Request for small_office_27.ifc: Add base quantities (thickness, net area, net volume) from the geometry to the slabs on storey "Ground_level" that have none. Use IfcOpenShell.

First a look at what the model holds.

```python
import ifcopenshell
import ifcopenshell.util.element
import ifcopenshell.util.unit

model = ifcopenshell.open("small_office_27.ifc")
print(model.schema)
for unit_type in ("LENGTHUNIT", "AREAUNIT", "VOLUMEUNIT"):
    print(unit_type, ifcopenshell.util.unit.calculate_unit_scale(model, unit_type))
storey = next(s for s in model.by_type("IfcBuildingStorey") if s.Name == "Ground_level")
slabs = [e for e in ifcopenshell.util.element.get_decomposition(storey) if e.is_a("IfcSlab")]
for e in sorted(slabs, key=lambda e: e.id()):
    print(e.id(), e.is_a(), e.Name, list(ifcopenshell.util.element.get_psets(e, qtos_only=True)), sep=" | ")
```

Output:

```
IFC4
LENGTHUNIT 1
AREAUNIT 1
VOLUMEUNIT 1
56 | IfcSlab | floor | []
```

```python
import ifcopenshell
import ifcopenshell.api.pset
import ifcopenshell.geom
import ifcopenshell.util.element
import ifcopenshell.util.shape
import ifcopenshell.util.unit

model = ifcopenshell.open("small_office_27.ifc")
unit_scale = ifcopenshell.util.unit.calculate_unit_scale(model)
area_scale = ifcopenshell.util.unit.calculate_unit_scale(model, "AREAUNIT")
volume_scale = ifcopenshell.util.unit.calculate_unit_scale(model, "VOLUMEUNIT")
settings = ifcopenshell.geom.settings()

storey = next(s for s in model.by_type("IfcBuildingStorey") if s.Name == "Ground_level")
slabs = [e for e in ifcopenshell.util.element.get_decomposition(storey) if e.is_a("IfcSlab")]

for e in sorted(slabs, key=lambda e: e.id()):
    if ifcopenshell.util.element.get_psets(e, qtos_only=True, should_inherit=False):
        continue
    # Geometry comes back in metres, in the element's own axes.
    shape = ifcopenshell.geom.create_shape(settings, e)
    values = {
        "Width": ifcopenshell.util.shape.get_z(shape.geometry) / unit_scale,
        "NetArea": ifcopenshell.util.shape.get_footprint_area(shape.geometry) / area_scale,
        "NetVolume": ifcopenshell.util.shape.get_volume(shape.geometry) / volume_scale,
    }
    qto = ifcopenshell.api.pset.add_qto(model, product=e, name="Qto_SlabBaseQuantities")
    ifcopenshell.api.pset.edit_qto(model, qto=qto, properties=values)
    print(e.id(), {k: round(v, 3) for k, v in values.items()})

model.write("small_office_27-out.ifc")
```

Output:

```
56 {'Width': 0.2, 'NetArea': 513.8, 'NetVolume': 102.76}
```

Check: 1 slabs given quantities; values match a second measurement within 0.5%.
